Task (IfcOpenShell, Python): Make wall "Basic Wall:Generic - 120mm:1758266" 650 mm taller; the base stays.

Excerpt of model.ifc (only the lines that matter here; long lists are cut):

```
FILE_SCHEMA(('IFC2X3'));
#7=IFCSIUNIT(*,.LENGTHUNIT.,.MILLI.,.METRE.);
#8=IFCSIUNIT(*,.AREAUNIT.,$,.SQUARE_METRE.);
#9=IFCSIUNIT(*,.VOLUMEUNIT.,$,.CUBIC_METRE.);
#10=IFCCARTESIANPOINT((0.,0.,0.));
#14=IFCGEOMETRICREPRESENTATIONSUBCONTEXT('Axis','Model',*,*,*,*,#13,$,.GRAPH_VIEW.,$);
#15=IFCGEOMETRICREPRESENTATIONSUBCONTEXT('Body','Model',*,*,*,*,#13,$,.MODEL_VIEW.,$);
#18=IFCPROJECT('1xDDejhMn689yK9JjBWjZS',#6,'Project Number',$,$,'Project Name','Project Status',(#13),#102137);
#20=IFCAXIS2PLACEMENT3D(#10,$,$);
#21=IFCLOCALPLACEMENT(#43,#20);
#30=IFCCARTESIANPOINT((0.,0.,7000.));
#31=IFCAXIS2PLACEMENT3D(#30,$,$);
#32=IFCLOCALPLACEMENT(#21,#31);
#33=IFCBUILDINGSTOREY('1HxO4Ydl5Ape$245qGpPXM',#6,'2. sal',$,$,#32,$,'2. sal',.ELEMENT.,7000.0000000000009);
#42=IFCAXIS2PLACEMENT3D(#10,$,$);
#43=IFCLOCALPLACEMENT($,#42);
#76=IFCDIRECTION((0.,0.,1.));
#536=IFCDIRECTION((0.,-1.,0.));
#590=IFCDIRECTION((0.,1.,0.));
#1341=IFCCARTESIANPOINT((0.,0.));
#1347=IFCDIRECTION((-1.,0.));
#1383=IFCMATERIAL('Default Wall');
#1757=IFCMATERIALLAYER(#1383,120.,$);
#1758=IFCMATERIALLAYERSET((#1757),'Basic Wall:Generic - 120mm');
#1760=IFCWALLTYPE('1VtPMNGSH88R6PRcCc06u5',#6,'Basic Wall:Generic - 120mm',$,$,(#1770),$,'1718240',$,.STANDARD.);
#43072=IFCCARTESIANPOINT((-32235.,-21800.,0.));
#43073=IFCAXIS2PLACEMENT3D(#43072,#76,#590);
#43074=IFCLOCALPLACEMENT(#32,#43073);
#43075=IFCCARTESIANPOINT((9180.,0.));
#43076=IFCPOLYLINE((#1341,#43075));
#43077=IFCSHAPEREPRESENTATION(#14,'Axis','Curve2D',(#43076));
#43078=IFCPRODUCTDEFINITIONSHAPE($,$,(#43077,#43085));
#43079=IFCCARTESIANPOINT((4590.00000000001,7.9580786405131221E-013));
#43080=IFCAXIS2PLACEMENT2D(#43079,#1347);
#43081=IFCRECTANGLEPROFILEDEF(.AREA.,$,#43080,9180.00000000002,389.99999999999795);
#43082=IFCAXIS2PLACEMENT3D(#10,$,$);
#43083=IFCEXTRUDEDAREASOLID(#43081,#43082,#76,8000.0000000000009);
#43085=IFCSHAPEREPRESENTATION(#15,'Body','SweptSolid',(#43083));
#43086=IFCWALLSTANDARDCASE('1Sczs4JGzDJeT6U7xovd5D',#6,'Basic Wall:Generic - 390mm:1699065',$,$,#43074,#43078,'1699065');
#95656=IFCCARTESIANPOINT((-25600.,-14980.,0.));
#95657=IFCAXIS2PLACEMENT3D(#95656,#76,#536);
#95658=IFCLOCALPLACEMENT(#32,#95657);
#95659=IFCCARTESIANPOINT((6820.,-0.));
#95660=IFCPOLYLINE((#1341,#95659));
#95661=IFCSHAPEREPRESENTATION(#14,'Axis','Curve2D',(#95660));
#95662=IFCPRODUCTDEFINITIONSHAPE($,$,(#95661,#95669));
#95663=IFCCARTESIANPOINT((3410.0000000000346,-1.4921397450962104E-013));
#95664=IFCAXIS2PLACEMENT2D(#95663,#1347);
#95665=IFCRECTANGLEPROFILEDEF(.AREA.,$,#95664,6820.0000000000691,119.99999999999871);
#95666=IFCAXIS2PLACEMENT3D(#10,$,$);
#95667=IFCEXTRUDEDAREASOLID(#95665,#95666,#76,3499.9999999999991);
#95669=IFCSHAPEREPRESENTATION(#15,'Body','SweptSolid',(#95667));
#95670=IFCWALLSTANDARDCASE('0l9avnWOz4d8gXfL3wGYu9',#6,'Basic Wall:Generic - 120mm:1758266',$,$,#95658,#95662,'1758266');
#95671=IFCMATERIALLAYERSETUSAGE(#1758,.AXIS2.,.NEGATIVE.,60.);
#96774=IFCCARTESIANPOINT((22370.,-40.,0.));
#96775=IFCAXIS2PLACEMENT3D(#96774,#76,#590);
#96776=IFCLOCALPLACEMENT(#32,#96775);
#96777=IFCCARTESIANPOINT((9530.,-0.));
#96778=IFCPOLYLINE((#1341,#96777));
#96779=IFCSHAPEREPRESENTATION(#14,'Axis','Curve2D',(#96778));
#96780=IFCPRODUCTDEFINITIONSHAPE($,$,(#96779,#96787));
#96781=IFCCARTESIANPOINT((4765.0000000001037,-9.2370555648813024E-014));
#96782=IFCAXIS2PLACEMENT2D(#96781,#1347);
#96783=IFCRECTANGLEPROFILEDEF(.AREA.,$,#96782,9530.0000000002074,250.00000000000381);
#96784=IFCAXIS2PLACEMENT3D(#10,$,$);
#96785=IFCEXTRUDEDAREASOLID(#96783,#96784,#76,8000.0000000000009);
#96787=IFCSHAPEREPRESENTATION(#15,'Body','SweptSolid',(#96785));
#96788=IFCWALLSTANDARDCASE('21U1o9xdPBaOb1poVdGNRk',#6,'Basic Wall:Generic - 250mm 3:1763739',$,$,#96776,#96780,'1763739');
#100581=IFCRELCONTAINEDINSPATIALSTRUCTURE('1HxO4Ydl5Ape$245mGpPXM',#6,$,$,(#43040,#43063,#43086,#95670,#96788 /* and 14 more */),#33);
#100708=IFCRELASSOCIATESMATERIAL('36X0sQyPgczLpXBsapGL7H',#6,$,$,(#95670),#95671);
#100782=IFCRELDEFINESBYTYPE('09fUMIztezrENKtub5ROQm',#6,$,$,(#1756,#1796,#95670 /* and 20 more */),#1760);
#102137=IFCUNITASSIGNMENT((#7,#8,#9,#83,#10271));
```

```python
import ifcopenshell
import ifcopenshell.geom
import ifcopenshell.util.representation
import ifcopenshell.util.shape
import ifcopenshell.util.unit

model = ifcopenshell.open("model.ifc")
unit_scale = ifcopenshell.util.unit.calculate_unit_scale(model)
settings = ifcopenshell.geom.settings()


def volume(element):
    """Net volume in cubic metres, openings subtracted."""
    shape = ifcopenshell.geom.create_shape(settings, element)
    return ifcopenshell.util.shape.get_volume(shape.geometry)


wall = model.by_id(95670)
before = volume(wall)

body = ifcopenshell.util.representation.get_representation(wall, "Model", "Body")
solid = body.Items[0]
old_height = solid.Depth
solid.Depth += 0.65 / unit_scale
after = volume(wall)

print(f"height {old_height:g} -> {solid.Depth:g}, volume {before:.3f} -> {after:.3f} m3")

model.write("model_rev.ifc")
```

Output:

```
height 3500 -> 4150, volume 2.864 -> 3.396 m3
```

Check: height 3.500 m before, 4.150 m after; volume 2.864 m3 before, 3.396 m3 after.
